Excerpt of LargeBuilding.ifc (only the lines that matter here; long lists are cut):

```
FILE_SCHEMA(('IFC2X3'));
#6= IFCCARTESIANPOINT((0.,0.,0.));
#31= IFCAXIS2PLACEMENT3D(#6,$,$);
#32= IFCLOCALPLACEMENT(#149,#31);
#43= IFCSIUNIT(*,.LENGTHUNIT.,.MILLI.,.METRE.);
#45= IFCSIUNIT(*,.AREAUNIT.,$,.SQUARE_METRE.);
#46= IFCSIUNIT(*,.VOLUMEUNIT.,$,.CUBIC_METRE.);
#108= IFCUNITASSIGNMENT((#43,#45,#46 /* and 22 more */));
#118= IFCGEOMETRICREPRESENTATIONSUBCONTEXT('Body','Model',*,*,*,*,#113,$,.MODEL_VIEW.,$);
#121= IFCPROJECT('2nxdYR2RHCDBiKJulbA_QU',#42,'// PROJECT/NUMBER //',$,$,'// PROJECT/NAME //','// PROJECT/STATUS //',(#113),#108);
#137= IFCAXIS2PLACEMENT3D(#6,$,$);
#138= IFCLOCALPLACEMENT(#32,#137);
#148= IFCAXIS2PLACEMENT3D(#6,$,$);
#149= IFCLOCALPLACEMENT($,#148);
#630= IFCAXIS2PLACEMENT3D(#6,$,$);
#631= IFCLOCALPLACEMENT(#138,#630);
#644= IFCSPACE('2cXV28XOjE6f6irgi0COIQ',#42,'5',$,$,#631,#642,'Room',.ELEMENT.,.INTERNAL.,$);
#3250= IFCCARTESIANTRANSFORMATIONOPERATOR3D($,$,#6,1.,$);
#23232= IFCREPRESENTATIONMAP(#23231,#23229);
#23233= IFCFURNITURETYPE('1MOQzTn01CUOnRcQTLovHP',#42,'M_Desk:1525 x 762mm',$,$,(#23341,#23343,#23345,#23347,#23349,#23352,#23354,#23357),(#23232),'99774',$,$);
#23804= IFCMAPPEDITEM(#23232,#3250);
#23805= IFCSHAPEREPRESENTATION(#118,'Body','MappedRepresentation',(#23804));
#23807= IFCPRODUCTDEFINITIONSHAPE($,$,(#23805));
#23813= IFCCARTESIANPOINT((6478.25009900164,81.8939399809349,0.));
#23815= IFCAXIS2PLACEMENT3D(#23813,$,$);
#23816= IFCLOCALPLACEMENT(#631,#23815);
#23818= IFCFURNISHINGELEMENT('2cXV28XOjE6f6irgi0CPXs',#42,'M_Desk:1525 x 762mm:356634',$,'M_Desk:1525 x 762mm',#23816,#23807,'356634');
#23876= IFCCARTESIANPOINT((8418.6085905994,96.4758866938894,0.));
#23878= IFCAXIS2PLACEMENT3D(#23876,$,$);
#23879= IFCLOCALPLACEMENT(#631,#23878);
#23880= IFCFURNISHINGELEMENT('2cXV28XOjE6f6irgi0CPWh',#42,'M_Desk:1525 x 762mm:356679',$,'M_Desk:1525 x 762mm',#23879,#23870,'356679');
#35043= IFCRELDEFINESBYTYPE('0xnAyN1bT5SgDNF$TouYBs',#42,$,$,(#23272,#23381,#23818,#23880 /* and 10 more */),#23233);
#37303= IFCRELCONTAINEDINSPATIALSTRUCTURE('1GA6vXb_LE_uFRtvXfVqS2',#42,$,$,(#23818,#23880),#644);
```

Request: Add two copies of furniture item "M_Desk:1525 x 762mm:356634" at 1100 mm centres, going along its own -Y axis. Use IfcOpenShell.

```python
import ifcopenshell
import ifcopenshell.api.geometry
import ifcopenshell.api.root
import ifcopenshell.util.element
import ifcopenshell.util.placement
import ifcopenshell.util.unit

model = ifcopenshell.open("LargeBuilding.ifc")
unit_scale = ifcopenshell.util.unit.calculate_unit_scale(model)


def reuse_history(source, copy):
    """copy_class also copies each property set's owner history, people and application; keep the originals."""
    for rel in copy.IsDefinedBy:
        if rel.is_a("IfcRelDefinesByProperties") and (history := rel.RelatingPropertyDefinition.OwnerHistory):
            rel.RelatingPropertyDefinition.OwnerHistory = source.OwnerHistory
            ifcopenshell.util.element.remove_deep2(model, history)


source = model.by_guid("2cXV28XOjE6f6irgi0CPXs")
base = ifcopenshell.util.placement.get_local_placement(source.ObjectPlacement)
step = -base[:3, 1] * 1.1 / unit_scale

for i in range(1, 3):
    copy = ifcopenshell.api.root.copy_class(model, product=source)
    copy.Representation = ifcopenshell.util.element.copy_deep(
        model, source.Representation, exclude=["IfcGeometricRepresentationContext", "IfcRepresentationMap"]
    )
    copy.Name = "M_Desk:1525 x 762mm"
    copy.Tag = None
    reuse_history(source, copy)
    matrix = base.copy()
    matrix[:3, 3] += i * step
    print("added at", matrix[:3, 3].round(3) + 0.0)
    ifcopenshell.api.geometry.edit_object_placement(model, product=copy, matrix=matrix, is_si=False)

model.write("LargeBuilding_v2.ifc")
```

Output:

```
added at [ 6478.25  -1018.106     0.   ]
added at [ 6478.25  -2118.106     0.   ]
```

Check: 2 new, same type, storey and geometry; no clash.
